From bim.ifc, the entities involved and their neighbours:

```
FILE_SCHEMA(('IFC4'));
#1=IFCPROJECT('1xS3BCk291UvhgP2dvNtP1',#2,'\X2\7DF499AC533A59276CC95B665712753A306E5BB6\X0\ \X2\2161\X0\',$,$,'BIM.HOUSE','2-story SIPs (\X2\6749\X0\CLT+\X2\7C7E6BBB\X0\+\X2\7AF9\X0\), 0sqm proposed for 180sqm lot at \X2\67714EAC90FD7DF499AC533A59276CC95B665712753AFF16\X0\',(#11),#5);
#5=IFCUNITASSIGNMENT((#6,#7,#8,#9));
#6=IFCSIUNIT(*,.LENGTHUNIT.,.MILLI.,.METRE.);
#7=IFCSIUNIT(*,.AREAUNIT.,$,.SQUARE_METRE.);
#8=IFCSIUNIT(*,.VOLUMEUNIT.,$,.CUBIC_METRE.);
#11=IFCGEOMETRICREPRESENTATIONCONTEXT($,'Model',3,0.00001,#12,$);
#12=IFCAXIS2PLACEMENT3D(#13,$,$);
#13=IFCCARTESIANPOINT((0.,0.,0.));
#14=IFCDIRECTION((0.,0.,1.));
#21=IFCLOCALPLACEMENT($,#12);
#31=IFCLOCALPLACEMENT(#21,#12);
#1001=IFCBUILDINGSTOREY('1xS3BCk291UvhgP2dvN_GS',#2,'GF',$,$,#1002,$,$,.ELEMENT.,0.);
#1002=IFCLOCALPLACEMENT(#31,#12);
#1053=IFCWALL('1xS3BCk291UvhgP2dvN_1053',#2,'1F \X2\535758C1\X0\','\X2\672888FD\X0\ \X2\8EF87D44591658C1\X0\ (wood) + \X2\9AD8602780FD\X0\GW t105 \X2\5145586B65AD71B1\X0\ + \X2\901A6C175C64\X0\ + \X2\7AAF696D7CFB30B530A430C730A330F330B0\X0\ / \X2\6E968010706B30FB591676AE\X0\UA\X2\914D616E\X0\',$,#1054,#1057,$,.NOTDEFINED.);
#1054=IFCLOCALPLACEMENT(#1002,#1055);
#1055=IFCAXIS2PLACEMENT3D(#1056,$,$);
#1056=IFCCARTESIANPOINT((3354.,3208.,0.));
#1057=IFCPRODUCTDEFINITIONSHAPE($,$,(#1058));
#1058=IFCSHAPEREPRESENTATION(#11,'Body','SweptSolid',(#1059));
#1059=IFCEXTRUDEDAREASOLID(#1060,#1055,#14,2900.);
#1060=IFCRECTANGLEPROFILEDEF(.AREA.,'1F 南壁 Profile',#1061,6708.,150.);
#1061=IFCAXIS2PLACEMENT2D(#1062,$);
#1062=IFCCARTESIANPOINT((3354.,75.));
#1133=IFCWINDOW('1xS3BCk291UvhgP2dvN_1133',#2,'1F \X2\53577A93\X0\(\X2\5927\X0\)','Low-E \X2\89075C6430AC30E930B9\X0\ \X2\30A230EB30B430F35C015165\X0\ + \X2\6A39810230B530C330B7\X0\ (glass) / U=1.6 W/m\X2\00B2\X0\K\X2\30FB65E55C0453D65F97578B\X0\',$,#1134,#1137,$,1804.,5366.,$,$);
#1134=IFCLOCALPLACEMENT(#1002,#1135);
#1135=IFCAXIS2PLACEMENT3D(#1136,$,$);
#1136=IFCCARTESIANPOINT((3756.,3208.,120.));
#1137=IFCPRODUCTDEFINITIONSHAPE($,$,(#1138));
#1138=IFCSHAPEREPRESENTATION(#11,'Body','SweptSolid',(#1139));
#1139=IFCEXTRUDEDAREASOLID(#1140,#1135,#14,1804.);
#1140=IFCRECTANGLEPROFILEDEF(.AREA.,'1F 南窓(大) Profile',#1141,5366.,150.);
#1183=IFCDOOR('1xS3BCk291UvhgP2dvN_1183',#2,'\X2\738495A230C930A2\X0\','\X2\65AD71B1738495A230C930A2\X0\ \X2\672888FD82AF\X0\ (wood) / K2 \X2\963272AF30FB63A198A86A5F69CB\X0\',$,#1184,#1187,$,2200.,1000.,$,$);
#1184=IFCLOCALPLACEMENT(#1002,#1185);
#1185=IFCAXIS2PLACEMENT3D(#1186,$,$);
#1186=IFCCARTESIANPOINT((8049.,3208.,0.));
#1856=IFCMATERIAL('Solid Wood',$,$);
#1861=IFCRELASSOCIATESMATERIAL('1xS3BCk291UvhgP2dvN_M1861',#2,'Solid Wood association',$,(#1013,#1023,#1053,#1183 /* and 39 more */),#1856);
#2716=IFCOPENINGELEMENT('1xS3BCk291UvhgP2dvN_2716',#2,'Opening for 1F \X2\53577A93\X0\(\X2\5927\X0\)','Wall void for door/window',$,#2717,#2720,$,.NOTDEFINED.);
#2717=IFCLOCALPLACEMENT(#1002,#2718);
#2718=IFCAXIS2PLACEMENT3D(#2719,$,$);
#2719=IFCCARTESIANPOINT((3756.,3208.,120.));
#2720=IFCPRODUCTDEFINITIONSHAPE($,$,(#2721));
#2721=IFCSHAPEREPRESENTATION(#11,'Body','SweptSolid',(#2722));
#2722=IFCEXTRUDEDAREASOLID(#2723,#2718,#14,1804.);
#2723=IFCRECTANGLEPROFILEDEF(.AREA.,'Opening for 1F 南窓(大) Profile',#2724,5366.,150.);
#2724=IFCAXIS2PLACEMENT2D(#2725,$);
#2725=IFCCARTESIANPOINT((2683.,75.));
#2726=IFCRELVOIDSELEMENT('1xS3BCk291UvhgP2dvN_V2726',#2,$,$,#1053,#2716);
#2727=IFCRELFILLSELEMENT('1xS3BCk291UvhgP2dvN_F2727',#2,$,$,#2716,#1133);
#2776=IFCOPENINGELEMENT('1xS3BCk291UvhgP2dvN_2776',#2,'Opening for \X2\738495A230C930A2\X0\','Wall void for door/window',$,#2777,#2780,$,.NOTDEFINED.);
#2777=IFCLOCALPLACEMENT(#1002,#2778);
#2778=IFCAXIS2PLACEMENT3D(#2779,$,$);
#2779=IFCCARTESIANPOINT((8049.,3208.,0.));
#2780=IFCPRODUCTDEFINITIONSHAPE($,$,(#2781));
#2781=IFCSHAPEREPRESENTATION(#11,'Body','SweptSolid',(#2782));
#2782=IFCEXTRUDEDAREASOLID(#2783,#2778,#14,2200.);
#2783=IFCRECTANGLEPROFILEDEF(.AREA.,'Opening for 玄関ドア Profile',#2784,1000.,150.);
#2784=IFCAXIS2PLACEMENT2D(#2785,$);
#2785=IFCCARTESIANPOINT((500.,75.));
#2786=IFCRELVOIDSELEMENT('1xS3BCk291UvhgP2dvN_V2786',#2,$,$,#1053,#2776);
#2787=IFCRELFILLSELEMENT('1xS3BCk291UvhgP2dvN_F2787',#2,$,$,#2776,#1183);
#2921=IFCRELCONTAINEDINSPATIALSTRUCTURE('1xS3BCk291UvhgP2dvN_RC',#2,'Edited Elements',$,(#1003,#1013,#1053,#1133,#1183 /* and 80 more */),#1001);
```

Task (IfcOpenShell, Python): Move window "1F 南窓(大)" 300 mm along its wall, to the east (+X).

```python
import ifcopenshell
import ifcopenshell.api.geometry
import ifcopenshell.util.placement

model = ifcopenshell.open("bim.ifc")

window = model.by_guid("1xS3BCk291UvhgP2dvN_1133")
opening = window.FillsVoids[0].RelatingOpeningElement
wall = opening.VoidsElements[0].RelatingBuildingElement

wall_matrix = ifcopenshell.util.placement.get_local_placement(wall.ObjectPlacement)
shift = wall_matrix[:3, 0] * 300.0
before = ifcopenshell.util.placement.get_local_placement(window.ObjectPlacement)[:3, 3].copy()

# The window is not placed relative to its opening, so move both.
for product in (opening, window):
    matrix = ifcopenshell.util.placement.get_local_placement(product.ObjectPlacement)
    matrix[:3, 3] += shift
    ifcopenshell.api.geometry.edit_object_placement(model, product=product, matrix=matrix, is_si=False)

after = ifcopenshell.util.placement.get_local_placement(window.ObjectPlacement)[:3, 3]
print("window moved by", (after - before).round(3) + 0.0)

model.write("bim_v2.ifc")
```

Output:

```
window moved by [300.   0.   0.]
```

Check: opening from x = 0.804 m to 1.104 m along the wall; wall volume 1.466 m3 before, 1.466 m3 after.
